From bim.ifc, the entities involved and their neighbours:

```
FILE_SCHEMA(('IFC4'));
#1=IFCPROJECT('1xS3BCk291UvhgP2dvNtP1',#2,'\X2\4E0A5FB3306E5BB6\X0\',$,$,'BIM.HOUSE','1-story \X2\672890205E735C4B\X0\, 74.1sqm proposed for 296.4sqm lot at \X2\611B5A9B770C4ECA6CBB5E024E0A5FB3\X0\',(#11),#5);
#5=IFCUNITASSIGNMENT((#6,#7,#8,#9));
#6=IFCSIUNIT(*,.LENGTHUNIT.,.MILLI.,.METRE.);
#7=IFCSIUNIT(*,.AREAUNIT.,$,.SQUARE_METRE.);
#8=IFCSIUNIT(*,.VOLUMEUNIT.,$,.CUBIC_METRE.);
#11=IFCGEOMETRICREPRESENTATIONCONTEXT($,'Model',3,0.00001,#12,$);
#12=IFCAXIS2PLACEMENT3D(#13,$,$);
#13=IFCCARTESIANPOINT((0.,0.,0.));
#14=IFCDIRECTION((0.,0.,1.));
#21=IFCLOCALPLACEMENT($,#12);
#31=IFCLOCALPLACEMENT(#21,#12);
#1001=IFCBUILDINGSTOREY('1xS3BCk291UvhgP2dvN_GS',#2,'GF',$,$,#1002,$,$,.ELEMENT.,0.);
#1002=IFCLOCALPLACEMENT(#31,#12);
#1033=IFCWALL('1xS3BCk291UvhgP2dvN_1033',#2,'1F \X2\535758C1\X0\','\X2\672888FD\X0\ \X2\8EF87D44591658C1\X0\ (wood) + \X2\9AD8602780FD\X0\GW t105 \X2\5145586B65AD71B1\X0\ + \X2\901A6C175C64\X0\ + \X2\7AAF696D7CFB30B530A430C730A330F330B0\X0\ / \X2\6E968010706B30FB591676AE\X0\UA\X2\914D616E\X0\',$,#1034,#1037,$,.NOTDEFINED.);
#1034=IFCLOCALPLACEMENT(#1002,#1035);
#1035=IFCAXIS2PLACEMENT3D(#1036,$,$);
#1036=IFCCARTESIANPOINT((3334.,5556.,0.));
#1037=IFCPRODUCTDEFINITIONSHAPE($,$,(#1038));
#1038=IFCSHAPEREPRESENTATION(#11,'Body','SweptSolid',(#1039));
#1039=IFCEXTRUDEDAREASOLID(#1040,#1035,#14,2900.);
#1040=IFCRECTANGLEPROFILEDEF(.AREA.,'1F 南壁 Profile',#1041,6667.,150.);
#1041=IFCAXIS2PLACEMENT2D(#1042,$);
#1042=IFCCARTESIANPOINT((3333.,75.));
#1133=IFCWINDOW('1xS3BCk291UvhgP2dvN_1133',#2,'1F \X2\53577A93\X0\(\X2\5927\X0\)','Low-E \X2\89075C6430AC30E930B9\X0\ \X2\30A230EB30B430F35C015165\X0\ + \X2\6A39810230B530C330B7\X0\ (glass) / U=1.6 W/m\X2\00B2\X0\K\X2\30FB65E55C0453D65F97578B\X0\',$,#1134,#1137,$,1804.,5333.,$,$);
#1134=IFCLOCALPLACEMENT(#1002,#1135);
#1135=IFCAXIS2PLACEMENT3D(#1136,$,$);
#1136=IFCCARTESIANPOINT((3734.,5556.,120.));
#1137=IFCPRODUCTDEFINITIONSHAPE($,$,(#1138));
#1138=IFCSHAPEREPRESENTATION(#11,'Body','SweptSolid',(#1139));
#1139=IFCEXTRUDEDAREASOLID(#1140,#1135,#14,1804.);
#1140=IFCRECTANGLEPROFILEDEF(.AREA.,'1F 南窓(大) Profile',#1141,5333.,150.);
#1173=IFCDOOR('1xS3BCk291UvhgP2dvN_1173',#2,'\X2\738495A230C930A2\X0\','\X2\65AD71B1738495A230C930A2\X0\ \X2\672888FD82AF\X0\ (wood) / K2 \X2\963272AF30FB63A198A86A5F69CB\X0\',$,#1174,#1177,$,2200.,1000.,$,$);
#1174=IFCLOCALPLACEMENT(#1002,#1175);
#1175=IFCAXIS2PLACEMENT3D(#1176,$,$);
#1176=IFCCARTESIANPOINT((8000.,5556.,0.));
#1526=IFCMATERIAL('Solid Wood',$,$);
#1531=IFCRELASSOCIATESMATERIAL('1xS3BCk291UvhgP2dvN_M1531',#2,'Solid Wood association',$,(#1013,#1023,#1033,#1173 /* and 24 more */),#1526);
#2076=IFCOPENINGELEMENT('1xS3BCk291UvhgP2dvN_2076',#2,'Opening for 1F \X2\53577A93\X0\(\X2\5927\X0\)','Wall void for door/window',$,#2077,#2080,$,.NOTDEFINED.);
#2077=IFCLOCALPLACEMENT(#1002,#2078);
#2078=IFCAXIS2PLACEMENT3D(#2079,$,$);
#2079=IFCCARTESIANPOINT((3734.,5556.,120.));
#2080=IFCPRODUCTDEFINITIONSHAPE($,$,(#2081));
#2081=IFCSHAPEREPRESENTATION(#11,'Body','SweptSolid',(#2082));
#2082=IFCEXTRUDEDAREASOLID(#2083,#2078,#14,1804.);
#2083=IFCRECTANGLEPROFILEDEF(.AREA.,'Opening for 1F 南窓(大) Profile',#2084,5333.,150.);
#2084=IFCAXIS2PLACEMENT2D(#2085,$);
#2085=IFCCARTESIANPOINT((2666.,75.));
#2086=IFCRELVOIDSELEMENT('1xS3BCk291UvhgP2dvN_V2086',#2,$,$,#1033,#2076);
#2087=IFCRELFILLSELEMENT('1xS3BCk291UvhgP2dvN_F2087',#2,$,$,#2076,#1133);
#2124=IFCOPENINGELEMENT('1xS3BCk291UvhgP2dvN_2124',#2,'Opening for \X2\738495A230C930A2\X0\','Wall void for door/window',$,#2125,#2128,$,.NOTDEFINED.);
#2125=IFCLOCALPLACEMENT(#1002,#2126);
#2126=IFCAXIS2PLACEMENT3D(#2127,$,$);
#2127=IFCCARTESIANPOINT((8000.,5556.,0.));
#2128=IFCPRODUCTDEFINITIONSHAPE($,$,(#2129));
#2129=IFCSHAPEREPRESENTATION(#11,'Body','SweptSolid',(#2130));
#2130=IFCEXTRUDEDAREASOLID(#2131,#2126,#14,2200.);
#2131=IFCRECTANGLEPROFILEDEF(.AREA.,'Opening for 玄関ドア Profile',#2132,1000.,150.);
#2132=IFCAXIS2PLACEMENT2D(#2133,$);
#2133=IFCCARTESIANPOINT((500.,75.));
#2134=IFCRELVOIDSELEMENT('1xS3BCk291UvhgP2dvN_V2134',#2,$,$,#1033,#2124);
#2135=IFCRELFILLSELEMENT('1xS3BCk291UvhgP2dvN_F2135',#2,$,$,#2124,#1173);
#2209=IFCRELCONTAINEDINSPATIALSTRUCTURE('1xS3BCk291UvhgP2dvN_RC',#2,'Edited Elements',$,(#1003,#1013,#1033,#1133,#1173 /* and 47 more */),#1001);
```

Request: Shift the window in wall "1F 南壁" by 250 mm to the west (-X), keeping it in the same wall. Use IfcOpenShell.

```python
import ifcopenshell
import ifcopenshell.api.geometry
import ifcopenshell.util.placement
import ifcopenshell.util.unit

model = ifcopenshell.open("bim.ifc")
unit_scale = ifcopenshell.util.unit.calculate_unit_scale(model)

window = model.by_guid("1xS3BCk291UvhgP2dvN_1133")
opening = window.FillsVoids[0].RelatingOpeningElement
wall = opening.VoidsElements[0].RelatingBuildingElement

wall_matrix = ifcopenshell.util.placement.get_local_placement(wall.ObjectPlacement)
shift = wall_matrix[:3, 0] * -0.25 / unit_scale
before = ifcopenshell.util.placement.get_local_placement(window.ObjectPlacement)[:3, 3].copy()

# The window is not placed relative to its opening, so move both.
for product in (opening, window):
    matrix = ifcopenshell.util.placement.get_local_placement(product.ObjectPlacement)
    matrix[:3, 3] += shift
    ifcopenshell.api.geometry.edit_object_placement(model, product=product, matrix=matrix, is_si=False)

after = ifcopenshell.util.placement.get_local_placement(window.ObjectPlacement)[:3, 3]
print("window moved by", (after - before).round(3) + 0.0)

model.write("bim_v2.ifc")
```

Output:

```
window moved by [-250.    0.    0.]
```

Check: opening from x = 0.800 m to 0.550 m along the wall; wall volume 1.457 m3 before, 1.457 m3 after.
